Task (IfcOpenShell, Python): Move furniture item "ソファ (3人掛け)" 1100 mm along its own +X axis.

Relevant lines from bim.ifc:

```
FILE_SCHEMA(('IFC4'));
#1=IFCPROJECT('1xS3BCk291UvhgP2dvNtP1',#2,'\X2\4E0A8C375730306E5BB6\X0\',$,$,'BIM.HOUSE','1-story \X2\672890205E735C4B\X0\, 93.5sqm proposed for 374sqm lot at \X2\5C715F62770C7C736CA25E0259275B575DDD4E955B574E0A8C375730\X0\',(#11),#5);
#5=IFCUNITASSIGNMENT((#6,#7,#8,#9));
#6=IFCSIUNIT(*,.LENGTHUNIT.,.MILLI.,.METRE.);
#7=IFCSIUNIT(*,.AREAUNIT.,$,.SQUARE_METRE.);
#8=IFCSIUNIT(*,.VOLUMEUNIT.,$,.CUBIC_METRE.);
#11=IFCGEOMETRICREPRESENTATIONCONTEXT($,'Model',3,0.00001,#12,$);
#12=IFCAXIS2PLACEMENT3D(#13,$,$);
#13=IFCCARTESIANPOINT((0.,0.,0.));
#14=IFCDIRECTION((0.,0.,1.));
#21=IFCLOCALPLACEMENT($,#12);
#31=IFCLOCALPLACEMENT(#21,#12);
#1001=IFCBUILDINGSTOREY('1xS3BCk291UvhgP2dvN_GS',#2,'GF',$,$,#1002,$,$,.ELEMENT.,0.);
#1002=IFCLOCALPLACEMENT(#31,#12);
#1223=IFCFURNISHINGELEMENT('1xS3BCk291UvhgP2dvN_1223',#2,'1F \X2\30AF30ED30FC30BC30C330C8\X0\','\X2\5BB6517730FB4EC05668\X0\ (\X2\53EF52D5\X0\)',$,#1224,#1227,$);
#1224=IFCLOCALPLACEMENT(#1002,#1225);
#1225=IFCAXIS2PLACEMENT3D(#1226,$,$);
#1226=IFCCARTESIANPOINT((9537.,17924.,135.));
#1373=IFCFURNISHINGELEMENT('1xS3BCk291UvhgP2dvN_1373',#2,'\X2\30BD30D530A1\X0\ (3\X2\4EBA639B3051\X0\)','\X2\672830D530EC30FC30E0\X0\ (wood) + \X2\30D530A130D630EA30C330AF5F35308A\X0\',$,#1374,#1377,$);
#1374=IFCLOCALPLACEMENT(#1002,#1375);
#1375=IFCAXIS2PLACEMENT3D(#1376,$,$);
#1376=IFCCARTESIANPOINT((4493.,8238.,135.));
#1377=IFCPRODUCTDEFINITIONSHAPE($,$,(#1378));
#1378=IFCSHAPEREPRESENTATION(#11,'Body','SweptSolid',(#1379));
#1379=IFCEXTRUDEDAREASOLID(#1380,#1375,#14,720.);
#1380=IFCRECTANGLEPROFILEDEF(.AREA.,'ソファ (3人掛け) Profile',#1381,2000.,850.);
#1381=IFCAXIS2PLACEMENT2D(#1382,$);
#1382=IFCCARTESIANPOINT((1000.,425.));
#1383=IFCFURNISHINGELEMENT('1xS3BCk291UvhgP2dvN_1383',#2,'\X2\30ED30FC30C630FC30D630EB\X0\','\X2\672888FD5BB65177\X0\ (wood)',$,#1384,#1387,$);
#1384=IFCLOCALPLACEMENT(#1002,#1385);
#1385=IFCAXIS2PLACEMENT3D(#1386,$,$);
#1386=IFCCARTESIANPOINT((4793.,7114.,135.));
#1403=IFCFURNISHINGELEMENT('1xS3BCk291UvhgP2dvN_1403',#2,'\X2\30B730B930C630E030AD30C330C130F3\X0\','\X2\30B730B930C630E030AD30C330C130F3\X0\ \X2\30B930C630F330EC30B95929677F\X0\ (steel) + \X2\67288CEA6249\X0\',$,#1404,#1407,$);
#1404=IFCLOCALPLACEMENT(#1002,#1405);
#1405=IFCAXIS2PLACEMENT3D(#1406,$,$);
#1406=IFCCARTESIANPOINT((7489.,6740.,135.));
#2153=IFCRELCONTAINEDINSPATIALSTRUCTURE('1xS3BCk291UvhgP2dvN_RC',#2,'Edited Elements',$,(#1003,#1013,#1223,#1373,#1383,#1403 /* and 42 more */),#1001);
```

```python
import ifcopenshell
import ifcopenshell.api.geometry
import ifcopenshell.util.placement
import ifcopenshell.util.unit

model = ifcopenshell.open("bim.ifc")
unit_scale = ifcopenshell.util.unit.calculate_unit_scale(model)

item = model.by_guid("1xS3BCk291UvhgP2dvN_1373")
matrix = ifcopenshell.util.placement.get_local_placement(item.ObjectPlacement)
matrix[:3, 3] += matrix[:3, 0] * 1.1 / unit_scale
ifcopenshell.api.geometry.edit_object_placement(model, product=item, matrix=matrix, is_si=False)

print(ifcopenshell.util.placement.get_local_placement(item.ObjectPlacement).round(3) + 0.0)

model.write("bim_updated.ifc")
```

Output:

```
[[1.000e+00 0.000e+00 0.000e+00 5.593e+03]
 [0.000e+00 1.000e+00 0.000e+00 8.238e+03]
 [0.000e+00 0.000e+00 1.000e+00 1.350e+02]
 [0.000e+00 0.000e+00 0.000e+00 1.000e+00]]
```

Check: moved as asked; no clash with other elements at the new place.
